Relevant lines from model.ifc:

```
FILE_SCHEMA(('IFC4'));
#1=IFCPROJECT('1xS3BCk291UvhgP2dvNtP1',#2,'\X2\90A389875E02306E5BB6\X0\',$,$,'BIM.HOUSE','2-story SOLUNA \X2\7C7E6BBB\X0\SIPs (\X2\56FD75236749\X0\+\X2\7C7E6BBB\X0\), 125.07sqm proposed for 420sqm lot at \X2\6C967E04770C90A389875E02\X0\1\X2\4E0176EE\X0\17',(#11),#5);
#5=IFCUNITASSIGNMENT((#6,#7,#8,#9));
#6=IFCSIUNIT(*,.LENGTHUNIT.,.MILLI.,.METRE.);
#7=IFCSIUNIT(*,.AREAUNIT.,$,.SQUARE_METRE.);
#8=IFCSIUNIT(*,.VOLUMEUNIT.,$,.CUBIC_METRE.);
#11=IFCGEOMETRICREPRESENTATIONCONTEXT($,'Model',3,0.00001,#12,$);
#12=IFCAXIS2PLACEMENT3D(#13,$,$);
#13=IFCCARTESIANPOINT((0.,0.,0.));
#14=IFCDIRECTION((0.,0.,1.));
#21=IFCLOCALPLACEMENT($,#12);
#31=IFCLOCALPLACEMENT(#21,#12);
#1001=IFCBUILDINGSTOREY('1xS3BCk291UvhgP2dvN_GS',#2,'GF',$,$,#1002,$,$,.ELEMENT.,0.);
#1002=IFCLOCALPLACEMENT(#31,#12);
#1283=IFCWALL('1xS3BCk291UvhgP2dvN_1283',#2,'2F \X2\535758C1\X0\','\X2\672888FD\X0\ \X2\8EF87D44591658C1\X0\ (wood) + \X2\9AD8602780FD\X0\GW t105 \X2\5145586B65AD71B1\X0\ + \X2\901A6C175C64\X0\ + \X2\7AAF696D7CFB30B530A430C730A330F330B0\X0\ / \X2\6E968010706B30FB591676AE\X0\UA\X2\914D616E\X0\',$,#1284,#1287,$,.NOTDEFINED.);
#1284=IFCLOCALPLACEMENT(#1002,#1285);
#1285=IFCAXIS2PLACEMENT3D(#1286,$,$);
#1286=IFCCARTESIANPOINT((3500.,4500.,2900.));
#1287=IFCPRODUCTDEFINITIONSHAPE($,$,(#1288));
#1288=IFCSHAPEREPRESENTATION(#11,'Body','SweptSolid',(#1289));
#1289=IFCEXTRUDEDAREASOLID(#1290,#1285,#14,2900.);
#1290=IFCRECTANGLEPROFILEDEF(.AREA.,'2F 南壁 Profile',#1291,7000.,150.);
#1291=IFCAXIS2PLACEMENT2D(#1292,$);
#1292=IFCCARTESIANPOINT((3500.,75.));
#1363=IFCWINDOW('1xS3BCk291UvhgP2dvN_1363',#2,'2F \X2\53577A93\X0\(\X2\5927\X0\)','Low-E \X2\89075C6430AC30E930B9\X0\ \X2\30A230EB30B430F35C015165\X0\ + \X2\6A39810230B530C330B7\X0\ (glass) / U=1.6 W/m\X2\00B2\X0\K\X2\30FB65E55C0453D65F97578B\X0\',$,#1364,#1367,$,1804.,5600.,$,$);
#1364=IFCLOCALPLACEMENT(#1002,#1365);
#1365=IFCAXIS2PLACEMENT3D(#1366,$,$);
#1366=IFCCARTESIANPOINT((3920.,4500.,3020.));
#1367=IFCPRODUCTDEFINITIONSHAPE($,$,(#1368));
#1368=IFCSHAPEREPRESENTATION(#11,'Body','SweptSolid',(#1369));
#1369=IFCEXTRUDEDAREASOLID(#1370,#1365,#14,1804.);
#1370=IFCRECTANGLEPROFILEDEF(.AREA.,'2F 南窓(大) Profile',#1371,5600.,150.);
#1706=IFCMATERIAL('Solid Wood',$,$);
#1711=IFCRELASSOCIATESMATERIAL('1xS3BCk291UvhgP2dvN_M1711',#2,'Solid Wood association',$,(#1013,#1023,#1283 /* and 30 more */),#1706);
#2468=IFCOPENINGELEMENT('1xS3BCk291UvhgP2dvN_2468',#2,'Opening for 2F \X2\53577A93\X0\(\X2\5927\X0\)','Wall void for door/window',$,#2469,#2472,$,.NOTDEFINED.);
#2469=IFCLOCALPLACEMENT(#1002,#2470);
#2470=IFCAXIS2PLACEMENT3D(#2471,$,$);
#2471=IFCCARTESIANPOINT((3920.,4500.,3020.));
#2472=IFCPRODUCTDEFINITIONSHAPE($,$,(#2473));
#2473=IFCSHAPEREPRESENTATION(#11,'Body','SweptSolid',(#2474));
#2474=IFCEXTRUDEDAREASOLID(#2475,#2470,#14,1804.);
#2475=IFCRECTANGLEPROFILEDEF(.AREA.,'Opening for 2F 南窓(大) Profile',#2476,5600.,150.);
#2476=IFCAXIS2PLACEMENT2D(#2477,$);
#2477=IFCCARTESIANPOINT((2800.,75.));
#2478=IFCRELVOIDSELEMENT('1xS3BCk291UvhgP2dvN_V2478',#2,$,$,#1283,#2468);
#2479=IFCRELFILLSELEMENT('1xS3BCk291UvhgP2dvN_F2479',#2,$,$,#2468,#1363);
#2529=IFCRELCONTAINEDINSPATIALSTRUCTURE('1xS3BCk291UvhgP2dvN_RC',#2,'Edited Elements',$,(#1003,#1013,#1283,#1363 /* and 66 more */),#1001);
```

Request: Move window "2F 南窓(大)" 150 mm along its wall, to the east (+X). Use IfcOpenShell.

```python
import ifcopenshell
import ifcopenshell.api.geometry
import ifcopenshell.util.placement
import ifcopenshell.util.unit

model = ifcopenshell.open("model.ifc")
unit_scale = ifcopenshell.util.unit.calculate_unit_scale(model)

window = model.by_guid("1xS3BCk291UvhgP2dvN_1363")
opening = window.FillsVoids[0].RelatingOpeningElement
wall = opening.VoidsElements[0].RelatingBuildingElement

wall_matrix = ifcopenshell.util.placement.get_local_placement(wall.ObjectPlacement)
shift = wall_matrix[:3, 0] * 0.15 / unit_scale
before = ifcopenshell.util.placement.get_local_placement(window.ObjectPlacement)[:3, 3].copy()

# The window is not placed relative to its opening, so move both.
for product in (opening, window):
    matrix = ifcopenshell.util.placement.get_local_placement(product.ObjectPlacement)
    matrix[:3, 3] += shift
    ifcopenshell.api.geometry.edit_object_placement(model, product=product, matrix=matrix, is_si=False)

after = ifcopenshell.util.placement.get_local_placement(window.ObjectPlacement)[:3, 3]
print("window moved by", (after - before).round(3) + 0.0)

model.write("model_updated.ifc")
```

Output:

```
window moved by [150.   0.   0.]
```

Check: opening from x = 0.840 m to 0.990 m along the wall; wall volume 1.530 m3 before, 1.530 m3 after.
